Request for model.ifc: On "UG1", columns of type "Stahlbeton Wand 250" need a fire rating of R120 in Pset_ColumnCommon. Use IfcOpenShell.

First a look at what the model holds.

```python
import ifcopenshell
import ifcopenshell.util.element

model = ifcopenshell.open("model.ifc")
print(model.schema)
storey = next(s for s in model.by_type("IfcBuildingStorey") if s.Name == "UG1")
columns = [e for e in ifcopenshell.util.element.get_decomposition(storey) if e.is_a("IfcColumn")]
seen = {}
for e in columns:
    element_type = ifcopenshell.util.element.get_type(e)
    key = (element_type.Name if element_type != e and element_type else None, ifcopenshell.util.element.get_pset(e, "Pset_ColumnCommon", "FireRating"))
    seen[key] = seen.get(key, 0) + 1
for (name, value), count in sorted(seen.items(), key=str):
    print(count, "x", name, "|", value)
```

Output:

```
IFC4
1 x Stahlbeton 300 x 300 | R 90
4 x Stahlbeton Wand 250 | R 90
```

```python
import ifcopenshell
import ifcopenshell.api.pset
import ifcopenshell.util.element

model = ifcopenshell.open("model.ifc")

storey = next(s for s in model.by_type("IfcBuildingStorey") if s.Name == "UG1")
columns = [e for e in ifcopenshell.util.element.get_decomposition(storey) if e.is_a("IfcColumn")]

count = 0
for e in columns:
    element_type = ifcopenshell.util.element.get_type(e)
    if element_type in (None, e) or element_type.Name != "Stahlbeton Wand 250":
        continue
    # add_pset returns the element's existing set when there is one.
    pset = ifcopenshell.api.pset.add_pset(model, product=e, name="Pset_ColumnCommon")
    ifcopenshell.api.pset.edit_pset(model, pset=pset, properties={"FireRating": "R120"})
    count += 1

print(count, "columns updated")

model.write("model_v2.ifc")
```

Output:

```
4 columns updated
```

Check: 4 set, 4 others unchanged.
